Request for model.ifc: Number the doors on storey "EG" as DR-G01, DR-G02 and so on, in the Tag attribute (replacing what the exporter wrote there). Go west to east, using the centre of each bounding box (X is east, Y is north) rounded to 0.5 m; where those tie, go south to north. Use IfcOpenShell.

First a look at what the model holds.

```python
import ifcopenshell
import ifcopenshell.util.element
import ifcopenshell.util.placement

model = ifcopenshell.open("model.ifc")
print(model.schema)
storey = next(s for s in model.by_type("IfcBuildingStorey") if s.Name == "EG")
doors = [e for e in ifcopenshell.util.element.get_decomposition(storey) if e.is_a("IfcDoor")]
for e in sorted(doors, key=lambda e: e.id()):
    origin = ifcopenshell.util.placement.get_local_placement(e.ObjectPlacement)[:3, 3]
    print(e.id(), e.Tag, e.Name, origin.round(2) + 0.0, sep=" | ")
```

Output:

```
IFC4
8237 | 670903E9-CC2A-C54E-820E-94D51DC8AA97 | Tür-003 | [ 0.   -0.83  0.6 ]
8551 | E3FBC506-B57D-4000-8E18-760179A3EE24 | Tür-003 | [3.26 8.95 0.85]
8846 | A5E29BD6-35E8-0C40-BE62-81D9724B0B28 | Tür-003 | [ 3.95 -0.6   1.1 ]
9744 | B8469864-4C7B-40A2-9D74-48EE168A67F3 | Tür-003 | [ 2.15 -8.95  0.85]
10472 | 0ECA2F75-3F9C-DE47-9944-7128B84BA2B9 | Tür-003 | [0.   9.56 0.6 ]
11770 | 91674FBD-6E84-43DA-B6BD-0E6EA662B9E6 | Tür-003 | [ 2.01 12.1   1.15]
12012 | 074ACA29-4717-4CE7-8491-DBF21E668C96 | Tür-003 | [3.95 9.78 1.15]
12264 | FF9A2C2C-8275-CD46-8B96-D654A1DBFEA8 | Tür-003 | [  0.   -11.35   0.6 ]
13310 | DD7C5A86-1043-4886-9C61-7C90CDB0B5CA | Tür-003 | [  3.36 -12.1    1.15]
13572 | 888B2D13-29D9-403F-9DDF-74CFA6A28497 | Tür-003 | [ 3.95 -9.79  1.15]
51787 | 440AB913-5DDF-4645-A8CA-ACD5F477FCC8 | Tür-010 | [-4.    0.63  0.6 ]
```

```python
import ifcopenshell
import ifcopenshell.geom
import ifcopenshell.util.element
import ifcopenshell.util.shape

model = ifcopenshell.open("model.ifc")
settings = ifcopenshell.geom.settings()
settings.set("use-world-coords", True)


def centre(element):
    shape = ifcopenshell.geom.create_shape(settings, element)
    return ifcopenshell.util.shape.get_bbox_centroid(shape.geometry)


storey = next(s for s in model.by_type("IfcBuildingStorey") if s.Name == "EG")
doors = [e for e in ifcopenshell.util.element.get_decomposition(storey) if e.is_a("IfcDoor")]

# Insertion points can sit at a corner or the storey origin, so sort by the geometry (in metres).
centres = {e: centre(e) for e in doors}
doors.sort(key=lambda e: (round(centres[e][0] / 0.5), centres[e][1]))

for i, e in enumerate(doors, start=1):
    number = f"DR-G{i:02d}"
    e.Tag = number
    print(e.id(), number)

model.write("model_edited.ifc")
```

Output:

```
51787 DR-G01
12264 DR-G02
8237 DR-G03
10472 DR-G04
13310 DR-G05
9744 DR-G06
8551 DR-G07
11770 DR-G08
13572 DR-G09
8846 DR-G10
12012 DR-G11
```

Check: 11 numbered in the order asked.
